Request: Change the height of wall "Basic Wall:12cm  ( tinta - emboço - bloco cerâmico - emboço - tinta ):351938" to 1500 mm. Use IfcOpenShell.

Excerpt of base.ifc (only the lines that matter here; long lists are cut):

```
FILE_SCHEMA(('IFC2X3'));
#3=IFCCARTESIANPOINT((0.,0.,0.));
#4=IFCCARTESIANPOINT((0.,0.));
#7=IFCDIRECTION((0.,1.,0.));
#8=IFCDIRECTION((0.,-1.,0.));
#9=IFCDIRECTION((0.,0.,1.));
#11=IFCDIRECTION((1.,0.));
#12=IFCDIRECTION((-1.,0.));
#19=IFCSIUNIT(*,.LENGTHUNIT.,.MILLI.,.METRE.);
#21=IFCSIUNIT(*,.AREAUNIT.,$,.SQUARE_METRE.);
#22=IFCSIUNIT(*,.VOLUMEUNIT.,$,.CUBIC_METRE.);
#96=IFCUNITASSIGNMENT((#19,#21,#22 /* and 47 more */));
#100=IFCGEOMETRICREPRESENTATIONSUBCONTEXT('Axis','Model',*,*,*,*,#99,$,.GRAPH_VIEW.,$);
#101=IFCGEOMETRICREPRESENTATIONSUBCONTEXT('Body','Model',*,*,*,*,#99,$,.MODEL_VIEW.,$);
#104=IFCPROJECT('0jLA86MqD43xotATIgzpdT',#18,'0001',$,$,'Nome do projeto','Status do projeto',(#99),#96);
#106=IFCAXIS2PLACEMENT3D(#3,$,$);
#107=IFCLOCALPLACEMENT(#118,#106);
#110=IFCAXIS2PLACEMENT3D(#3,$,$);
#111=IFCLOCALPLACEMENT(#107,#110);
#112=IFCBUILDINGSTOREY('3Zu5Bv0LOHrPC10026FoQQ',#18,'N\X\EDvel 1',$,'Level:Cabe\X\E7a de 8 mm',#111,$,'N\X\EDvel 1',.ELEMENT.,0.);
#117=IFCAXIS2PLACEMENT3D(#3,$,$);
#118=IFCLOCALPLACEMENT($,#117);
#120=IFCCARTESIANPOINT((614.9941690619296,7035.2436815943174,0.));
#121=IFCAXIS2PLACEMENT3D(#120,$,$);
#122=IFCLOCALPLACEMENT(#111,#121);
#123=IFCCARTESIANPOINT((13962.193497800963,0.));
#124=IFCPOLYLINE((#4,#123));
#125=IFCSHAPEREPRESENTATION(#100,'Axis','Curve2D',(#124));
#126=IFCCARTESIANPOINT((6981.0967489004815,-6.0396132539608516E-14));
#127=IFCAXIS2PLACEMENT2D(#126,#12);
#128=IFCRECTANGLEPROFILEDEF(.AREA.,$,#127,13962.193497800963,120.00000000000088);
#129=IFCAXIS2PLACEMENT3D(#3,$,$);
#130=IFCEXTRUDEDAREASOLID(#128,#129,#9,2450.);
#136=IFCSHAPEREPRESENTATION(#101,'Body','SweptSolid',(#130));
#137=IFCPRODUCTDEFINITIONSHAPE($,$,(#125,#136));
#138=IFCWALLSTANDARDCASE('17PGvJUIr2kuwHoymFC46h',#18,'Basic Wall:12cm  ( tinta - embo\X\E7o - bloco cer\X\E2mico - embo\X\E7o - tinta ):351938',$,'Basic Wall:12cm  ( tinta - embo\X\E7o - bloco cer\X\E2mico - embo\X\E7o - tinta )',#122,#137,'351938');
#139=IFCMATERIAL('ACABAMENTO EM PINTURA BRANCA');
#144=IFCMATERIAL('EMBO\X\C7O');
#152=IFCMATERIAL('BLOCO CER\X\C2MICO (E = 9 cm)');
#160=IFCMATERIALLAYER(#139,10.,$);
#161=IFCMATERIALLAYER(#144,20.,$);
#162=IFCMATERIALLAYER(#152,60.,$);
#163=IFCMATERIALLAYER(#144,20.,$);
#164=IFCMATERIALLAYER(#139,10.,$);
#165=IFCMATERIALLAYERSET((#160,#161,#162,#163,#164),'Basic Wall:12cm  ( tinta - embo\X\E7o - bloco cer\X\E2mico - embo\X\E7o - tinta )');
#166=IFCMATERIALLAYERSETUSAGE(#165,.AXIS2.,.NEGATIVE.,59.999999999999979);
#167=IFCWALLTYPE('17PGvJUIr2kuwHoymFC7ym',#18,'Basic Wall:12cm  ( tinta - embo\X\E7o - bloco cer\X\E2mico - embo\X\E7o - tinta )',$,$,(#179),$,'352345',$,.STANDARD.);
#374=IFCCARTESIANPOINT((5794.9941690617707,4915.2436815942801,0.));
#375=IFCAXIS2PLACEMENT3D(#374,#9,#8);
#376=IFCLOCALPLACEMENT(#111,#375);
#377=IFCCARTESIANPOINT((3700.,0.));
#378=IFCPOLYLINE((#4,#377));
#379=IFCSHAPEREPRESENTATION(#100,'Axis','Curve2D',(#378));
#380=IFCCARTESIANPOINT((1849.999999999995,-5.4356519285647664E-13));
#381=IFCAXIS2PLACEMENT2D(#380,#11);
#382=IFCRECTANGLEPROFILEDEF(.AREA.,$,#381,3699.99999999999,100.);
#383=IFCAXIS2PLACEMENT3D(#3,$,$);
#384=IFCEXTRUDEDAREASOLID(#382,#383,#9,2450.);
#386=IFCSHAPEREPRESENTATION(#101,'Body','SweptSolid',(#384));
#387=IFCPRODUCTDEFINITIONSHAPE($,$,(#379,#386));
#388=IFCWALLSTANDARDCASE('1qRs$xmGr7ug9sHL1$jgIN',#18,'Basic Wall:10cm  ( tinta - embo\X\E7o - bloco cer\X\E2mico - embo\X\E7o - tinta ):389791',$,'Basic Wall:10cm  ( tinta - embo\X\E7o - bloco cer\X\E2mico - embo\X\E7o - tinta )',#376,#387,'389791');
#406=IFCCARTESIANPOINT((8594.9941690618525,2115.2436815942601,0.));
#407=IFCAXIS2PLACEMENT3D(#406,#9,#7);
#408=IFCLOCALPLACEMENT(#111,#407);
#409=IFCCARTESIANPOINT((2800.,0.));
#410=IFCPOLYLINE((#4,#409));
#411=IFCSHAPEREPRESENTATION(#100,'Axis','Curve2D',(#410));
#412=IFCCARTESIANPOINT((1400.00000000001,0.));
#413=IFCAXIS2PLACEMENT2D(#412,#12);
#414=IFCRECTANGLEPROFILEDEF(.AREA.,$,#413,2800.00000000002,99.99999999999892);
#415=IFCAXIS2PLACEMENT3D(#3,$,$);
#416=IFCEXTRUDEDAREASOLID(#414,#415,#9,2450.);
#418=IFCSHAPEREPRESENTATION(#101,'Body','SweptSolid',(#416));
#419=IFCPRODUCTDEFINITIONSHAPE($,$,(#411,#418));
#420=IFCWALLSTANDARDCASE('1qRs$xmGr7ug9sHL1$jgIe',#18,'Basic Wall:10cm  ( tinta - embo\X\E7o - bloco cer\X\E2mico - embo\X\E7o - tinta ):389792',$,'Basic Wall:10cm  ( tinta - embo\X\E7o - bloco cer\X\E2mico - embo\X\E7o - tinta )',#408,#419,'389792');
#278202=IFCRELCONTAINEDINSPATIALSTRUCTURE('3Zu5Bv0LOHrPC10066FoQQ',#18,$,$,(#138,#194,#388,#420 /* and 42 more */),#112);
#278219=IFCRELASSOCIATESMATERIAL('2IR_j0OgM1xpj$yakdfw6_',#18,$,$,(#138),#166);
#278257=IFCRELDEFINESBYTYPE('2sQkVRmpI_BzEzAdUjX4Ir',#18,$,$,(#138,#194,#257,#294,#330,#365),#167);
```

```python
import ifcopenshell
import ifcopenshell.geom
import ifcopenshell.util.representation
import ifcopenshell.util.shape

model = ifcopenshell.open("base.ifc")
settings = ifcopenshell.geom.settings()


def volume(element):
    """Net volume in cubic metres, openings subtracted."""
    shape = ifcopenshell.geom.create_shape(settings, element)
    return ifcopenshell.util.shape.get_volume(shape.geometry)


wall = model.by_id(138)
before = volume(wall)

body = ifcopenshell.util.representation.get_representation(wall, "Model", "Body")
solid = body.Items[0]
old_height = solid.Depth
solid.Depth = 1500.0
after = volume(wall)

print(f"height {old_height:g} -> {solid.Depth:g}, volume {before:.3f} -> {after:.3f} m3")

model.write("base_rev.ifc")
```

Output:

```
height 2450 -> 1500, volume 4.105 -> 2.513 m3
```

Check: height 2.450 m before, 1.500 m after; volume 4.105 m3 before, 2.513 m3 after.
